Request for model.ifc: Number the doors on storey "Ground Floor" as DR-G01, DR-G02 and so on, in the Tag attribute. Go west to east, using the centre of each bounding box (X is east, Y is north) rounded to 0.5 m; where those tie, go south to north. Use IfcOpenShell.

First a look at what the model holds.

```python
import ifcopenshell
import ifcopenshell.util.element
import ifcopenshell.util.placement

model = ifcopenshell.open("model.ifc")
print(model.schema)
storey = next(s for s in model.by_type("IfcBuildingStorey") if s.Name == "Ground Floor")
doors = [e for e in ifcopenshell.util.element.get_decomposition(storey) if e.is_a("IfcDoor")]
for e in sorted(doors, key=lambda e: e.id()):
    origin = ifcopenshell.util.placement.get_local_placement(e.ObjectPlacement)[:3, 3]
    print(e.id(), e.Tag, e.Name, origin.round(2) + 0.0, sep=" | ")
```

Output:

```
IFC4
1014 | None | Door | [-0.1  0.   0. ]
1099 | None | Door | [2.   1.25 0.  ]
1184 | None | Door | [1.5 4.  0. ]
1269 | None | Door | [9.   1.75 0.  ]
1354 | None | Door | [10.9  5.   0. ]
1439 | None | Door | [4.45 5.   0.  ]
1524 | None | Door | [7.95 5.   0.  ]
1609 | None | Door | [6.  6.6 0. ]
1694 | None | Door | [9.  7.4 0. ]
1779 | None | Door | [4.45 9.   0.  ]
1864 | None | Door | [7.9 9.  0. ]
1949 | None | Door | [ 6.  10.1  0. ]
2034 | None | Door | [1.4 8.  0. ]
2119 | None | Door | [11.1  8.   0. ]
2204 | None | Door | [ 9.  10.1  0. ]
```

```python
import ifcopenshell
import ifcopenshell.geom
import ifcopenshell.util.element
import ifcopenshell.util.shape

model = ifcopenshell.open("model.ifc")
settings = ifcopenshell.geom.settings()
settings.set("use-world-coords", True)


def centre(element):
    shape = ifcopenshell.geom.create_shape(settings, element)
    return ifcopenshell.util.shape.get_bbox_centroid(shape.geometry)


storey = next(s for s in model.by_type("IfcBuildingStorey") if s.Name == "Ground Floor")
doors = [e for e in ifcopenshell.util.element.get_decomposition(storey) if e.is_a("IfcDoor")]

# Insertion points can sit at a corner or the storey origin, so sort by the geometry (in metres).
centres = {e: centre(e) for e in doors}
doors.sort(key=lambda e: (round(centres[e][0] / 0.5), centres[e][1]))

for i, e in enumerate(doors, start=1):
    number = f"DR-G{i:02d}"
    e.Tag = number
    print(e.id(), number)

model.write("model_updated.ifc")
```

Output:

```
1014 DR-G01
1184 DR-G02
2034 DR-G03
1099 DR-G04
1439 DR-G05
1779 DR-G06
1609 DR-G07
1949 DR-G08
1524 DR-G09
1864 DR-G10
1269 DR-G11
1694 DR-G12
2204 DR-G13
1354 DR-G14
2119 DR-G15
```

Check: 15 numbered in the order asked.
